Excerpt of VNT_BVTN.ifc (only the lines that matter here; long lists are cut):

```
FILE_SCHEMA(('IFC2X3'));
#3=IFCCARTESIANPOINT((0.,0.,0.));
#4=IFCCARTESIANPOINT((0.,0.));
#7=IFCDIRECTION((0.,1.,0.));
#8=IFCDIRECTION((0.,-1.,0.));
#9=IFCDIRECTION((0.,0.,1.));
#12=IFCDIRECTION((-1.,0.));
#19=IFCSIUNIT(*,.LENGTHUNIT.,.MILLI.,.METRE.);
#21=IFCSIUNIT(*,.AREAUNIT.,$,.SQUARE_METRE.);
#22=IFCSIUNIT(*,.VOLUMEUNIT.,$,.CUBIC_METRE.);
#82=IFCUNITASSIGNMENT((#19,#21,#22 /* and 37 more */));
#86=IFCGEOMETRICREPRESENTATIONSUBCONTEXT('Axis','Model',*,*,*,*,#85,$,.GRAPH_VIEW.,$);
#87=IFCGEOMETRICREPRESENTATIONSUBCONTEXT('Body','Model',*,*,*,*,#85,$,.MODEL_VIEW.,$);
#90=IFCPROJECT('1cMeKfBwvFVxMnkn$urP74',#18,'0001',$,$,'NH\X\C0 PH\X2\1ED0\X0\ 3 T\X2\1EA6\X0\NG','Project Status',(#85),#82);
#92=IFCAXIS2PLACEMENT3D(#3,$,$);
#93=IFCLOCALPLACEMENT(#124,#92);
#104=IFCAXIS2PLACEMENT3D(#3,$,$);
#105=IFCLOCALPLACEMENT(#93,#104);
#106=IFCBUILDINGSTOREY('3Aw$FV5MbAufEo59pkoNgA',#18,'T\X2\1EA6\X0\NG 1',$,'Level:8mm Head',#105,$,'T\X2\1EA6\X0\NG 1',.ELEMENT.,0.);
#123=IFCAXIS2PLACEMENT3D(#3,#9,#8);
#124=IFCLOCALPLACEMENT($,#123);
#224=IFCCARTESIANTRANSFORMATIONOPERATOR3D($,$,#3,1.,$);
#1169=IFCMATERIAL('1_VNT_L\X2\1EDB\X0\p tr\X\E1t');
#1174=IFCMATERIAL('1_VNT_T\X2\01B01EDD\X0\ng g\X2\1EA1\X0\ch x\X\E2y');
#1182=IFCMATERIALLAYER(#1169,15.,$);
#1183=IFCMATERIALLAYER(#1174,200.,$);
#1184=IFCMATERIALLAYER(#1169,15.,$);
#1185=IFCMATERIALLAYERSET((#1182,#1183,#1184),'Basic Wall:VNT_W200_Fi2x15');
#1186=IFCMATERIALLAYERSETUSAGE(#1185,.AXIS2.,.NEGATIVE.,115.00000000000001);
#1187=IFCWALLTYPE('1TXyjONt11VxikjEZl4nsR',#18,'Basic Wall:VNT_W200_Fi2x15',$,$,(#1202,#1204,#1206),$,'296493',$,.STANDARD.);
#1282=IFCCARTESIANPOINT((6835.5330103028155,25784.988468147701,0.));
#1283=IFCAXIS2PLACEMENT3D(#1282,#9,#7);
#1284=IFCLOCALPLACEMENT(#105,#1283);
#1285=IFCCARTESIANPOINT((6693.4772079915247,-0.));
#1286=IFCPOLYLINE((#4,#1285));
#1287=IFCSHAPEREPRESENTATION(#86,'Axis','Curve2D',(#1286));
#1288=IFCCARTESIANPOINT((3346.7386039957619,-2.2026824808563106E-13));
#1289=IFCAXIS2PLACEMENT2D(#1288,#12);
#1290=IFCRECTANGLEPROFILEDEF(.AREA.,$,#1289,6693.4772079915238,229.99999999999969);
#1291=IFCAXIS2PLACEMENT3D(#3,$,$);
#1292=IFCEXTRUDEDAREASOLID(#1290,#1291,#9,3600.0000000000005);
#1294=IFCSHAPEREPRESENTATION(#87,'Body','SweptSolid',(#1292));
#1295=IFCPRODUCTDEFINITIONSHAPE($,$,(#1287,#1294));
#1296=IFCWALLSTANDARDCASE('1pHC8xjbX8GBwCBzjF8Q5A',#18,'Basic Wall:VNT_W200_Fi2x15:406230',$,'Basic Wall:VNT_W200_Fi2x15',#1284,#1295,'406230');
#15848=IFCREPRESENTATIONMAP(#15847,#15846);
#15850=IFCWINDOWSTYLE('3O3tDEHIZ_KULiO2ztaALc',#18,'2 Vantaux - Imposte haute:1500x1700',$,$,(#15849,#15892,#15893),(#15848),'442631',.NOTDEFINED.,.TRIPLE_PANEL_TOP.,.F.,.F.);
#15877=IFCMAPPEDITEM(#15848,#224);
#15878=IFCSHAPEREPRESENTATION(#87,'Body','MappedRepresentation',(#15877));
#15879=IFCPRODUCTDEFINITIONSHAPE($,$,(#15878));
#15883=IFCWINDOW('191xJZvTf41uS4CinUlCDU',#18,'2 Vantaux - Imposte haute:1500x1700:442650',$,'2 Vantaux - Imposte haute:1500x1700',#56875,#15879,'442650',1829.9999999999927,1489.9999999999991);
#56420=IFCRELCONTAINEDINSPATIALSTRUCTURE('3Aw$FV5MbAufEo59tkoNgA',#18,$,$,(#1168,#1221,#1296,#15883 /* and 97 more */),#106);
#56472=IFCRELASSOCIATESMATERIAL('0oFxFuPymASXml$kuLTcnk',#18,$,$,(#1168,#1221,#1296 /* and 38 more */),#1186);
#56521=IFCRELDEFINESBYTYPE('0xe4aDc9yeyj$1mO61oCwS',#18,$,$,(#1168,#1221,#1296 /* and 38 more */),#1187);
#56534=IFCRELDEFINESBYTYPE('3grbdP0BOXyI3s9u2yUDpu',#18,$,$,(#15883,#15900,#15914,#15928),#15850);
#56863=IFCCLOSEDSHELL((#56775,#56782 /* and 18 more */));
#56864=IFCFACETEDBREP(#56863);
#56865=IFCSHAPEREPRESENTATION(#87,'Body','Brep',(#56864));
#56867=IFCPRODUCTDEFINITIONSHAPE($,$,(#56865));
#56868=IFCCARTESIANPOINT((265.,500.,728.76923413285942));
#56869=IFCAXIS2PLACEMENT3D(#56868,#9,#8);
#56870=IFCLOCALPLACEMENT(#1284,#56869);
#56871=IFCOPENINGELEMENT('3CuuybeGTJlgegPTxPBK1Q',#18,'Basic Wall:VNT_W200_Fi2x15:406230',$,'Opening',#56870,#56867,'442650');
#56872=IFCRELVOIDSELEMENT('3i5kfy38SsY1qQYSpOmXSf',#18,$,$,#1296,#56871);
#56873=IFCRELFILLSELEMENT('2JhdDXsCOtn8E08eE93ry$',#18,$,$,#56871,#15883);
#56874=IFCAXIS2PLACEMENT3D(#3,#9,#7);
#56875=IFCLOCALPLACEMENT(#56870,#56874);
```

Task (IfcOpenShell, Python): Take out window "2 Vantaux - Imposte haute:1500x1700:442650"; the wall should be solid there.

```python
import ifcopenshell
import ifcopenshell.api.feature
import ifcopenshell.api.root
import ifcopenshell.geom
import ifcopenshell.util.shape

model = ifcopenshell.open("VNT_BVTN.ifc")
settings = ifcopenshell.geom.settings()


def volume(element):
    """Net volume in cubic metres, openings subtracted."""
    shape = ifcopenshell.geom.create_shape(settings, element)
    return ifcopenshell.util.shape.get_volume(shape.geometry)


window = model.by_guid("191xJZvTf41uS4CinUlCDU")
opening = window.FillsVoids[0].RelatingOpeningElement
wall = opening.VoidsElements[0].RelatingBuildingElement
before = volume(wall)

ifcopenshell.api.root.remove_product(model, product=window)
ifcopenshell.api.feature.remove_feature(model, feature=opening)

after = volume(wall)

print(f"wall volume {before:.3f} -> {after:.3f} m3")

model.write("VNT_BVTN_edited.ifc")
```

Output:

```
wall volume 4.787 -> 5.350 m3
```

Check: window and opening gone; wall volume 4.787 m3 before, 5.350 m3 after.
